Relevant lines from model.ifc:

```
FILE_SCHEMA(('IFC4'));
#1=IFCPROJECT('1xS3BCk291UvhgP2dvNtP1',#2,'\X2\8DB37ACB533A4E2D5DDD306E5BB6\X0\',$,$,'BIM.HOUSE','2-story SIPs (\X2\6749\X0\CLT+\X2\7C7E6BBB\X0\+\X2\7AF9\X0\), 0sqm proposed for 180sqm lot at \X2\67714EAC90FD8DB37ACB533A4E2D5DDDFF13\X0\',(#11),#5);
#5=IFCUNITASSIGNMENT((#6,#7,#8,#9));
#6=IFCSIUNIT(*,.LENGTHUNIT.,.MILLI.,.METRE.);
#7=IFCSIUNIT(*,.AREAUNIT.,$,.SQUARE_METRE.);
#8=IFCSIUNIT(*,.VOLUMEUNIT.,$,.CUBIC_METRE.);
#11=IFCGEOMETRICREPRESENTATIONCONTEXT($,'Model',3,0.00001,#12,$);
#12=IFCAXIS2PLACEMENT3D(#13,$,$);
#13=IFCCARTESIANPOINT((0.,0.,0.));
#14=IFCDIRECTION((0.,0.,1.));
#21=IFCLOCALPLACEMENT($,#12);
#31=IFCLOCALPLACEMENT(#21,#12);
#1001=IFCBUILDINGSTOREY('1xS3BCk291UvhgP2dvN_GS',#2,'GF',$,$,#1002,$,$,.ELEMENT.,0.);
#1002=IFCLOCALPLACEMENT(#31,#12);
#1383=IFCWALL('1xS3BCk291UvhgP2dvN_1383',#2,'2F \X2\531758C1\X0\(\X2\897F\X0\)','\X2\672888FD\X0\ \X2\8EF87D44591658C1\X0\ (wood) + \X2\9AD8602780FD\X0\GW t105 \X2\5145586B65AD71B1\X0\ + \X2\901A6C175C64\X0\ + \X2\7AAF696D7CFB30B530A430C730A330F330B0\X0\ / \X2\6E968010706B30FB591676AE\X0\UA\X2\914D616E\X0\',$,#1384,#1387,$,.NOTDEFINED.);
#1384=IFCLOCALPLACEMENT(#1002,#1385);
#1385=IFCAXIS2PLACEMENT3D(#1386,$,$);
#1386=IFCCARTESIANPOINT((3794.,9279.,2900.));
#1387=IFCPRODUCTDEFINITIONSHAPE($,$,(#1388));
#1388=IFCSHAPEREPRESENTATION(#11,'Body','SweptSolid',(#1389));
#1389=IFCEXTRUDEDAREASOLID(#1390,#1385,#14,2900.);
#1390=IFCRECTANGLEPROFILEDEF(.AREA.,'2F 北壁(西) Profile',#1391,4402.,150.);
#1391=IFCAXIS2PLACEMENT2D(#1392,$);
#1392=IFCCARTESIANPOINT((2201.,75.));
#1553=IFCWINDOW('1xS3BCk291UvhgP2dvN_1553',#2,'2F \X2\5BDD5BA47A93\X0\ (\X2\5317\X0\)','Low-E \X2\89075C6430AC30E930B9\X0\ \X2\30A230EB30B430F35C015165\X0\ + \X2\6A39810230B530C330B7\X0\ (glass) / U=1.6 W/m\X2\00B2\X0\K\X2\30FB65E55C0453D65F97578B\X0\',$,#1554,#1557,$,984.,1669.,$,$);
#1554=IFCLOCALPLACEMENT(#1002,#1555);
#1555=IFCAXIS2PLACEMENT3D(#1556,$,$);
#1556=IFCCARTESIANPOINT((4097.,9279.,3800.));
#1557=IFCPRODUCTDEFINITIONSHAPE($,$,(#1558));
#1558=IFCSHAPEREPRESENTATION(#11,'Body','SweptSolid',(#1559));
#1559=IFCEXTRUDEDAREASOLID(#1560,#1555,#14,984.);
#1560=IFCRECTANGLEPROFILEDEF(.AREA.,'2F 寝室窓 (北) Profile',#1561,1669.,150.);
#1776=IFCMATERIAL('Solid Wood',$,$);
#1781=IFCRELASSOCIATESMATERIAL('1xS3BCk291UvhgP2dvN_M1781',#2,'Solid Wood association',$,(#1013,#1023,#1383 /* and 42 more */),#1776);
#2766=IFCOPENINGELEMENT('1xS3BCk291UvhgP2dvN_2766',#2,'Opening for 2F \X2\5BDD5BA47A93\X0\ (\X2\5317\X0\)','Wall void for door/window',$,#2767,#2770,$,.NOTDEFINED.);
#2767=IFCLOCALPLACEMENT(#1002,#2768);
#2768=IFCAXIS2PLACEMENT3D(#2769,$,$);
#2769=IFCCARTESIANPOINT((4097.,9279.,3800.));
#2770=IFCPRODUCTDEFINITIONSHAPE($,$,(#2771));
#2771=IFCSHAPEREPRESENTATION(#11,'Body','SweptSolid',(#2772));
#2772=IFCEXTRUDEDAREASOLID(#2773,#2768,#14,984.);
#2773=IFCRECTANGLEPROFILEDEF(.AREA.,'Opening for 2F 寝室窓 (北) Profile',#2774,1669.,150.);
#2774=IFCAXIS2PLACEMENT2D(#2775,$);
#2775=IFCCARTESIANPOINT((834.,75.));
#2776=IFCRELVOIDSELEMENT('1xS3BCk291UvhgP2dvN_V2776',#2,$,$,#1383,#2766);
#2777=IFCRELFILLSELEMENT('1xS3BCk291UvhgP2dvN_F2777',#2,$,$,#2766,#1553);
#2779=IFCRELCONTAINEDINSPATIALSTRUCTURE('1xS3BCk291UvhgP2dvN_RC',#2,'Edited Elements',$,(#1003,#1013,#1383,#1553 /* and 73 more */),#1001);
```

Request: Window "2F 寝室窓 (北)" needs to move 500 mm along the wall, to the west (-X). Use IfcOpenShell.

```python
import ifcopenshell
import ifcopenshell.api.geometry
import ifcopenshell.util.placement
import ifcopenshell.util.unit

model = ifcopenshell.open("model.ifc")
unit_scale = ifcopenshell.util.unit.calculate_unit_scale(model)

window = model.by_id(1553)
opening = window.FillsVoids[0].RelatingOpeningElement
wall = opening.VoidsElements[0].RelatingBuildingElement

wall_matrix = ifcopenshell.util.placement.get_local_placement(wall.ObjectPlacement)
shift = wall_matrix[:3, 0] * -0.5 / unit_scale
before = ifcopenshell.util.placement.get_local_placement(window.ObjectPlacement)[:3, 3].copy()

# The window is not placed relative to its opening, so move both.
for product in (opening, window):
    matrix = ifcopenshell.util.placement.get_local_placement(product.ObjectPlacement)
    matrix[:3, 3] += shift
    ifcopenshell.api.geometry.edit_object_placement(model, product=product, matrix=matrix, is_si=False)

after = ifcopenshell.util.placement.get_local_placement(window.ObjectPlacement)[:3, 3]
print("window moved by", (after - before).round(3) + 0.0)

model.write("model_updated.ifc")
```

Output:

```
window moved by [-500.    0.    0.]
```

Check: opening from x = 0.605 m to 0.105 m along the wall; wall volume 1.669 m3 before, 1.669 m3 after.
